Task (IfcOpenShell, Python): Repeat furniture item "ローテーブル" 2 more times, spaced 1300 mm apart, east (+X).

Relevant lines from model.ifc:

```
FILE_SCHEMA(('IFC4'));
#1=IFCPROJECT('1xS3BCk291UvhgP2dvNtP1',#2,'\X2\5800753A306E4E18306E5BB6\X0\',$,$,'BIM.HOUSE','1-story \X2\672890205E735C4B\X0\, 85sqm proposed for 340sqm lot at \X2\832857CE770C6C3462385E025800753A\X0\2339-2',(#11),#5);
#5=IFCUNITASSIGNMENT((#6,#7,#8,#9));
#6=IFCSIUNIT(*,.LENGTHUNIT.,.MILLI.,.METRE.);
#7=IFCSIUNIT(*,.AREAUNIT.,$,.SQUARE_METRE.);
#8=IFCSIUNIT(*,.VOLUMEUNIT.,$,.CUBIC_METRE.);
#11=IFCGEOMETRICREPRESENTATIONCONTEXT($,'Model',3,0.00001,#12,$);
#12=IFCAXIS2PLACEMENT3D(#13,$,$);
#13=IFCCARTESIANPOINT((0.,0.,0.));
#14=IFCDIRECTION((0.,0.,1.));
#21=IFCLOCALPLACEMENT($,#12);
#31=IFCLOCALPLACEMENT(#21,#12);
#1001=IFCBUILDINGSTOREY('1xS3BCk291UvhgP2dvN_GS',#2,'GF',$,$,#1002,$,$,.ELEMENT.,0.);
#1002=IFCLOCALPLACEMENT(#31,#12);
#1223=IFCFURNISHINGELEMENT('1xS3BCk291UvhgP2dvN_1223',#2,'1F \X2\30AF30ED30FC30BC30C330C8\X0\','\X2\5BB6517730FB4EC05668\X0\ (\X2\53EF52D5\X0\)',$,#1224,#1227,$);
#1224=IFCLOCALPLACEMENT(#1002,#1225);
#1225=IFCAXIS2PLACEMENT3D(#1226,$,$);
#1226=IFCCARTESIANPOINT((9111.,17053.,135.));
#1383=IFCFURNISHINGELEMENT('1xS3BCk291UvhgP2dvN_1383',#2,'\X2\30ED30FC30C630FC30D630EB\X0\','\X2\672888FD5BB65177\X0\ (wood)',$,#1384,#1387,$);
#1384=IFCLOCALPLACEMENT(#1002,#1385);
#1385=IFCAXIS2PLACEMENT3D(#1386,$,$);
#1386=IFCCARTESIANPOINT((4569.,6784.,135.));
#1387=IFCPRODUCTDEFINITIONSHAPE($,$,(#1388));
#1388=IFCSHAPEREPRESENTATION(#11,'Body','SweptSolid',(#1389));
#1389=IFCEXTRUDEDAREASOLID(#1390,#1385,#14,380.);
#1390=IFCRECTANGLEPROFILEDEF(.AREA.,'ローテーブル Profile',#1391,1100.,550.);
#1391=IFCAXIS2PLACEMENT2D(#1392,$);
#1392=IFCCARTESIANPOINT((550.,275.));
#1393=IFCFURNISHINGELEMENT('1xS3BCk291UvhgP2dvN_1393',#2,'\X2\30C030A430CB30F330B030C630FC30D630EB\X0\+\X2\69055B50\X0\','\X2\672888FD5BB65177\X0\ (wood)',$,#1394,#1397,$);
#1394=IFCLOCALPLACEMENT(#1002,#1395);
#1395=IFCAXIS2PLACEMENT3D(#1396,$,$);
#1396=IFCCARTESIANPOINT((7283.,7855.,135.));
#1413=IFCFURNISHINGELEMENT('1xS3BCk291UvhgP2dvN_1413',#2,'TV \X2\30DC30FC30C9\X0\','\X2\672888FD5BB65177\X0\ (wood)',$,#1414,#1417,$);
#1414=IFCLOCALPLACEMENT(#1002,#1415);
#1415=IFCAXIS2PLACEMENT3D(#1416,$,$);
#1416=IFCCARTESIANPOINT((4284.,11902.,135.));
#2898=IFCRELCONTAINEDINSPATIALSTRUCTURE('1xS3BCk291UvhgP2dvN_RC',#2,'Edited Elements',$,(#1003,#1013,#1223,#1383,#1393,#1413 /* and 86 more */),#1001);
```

```python
import numpy as np
import ifcopenshell
import ifcopenshell.api.geometry
import ifcopenshell.api.root
import ifcopenshell.util.element
import ifcopenshell.util.placement

model = ifcopenshell.open("model.ifc")


def reuse_history(source, copy):
    """copy_class also copies each property set's owner history, people and application; keep the originals."""
    for rel in copy.IsDefinedBy:
        if rel.is_a("IfcRelDefinesByProperties") and (history := rel.RelatingPropertyDefinition.OwnerHistory):
            rel.RelatingPropertyDefinition.OwnerHistory = source.OwnerHistory
            ifcopenshell.util.element.remove_deep2(model, history)


source = model.by_guid("1xS3BCk291UvhgP2dvN_1383")
base = ifcopenshell.util.placement.get_local_placement(source.ObjectPlacement)
step = np.array([1.0, 0.0, 0.0]) * 1300.0

for i in range(1, 3):
    copy = ifcopenshell.api.root.copy_class(model, product=source)
    copy.Representation = ifcopenshell.util.element.copy_deep(
        model, source.Representation, exclude=["IfcGeometricRepresentationContext", "IfcRepresentationMap"]
    )
    reuse_history(source, copy)
    matrix = base.copy()
    matrix[:3, 3] += i * step
    print("added at", matrix[:3, 3].round(3) + 0.0)
    ifcopenshell.api.geometry.edit_object_placement(model, product=copy, matrix=matrix, is_si=False)

model.write("model_rev.ifc")
```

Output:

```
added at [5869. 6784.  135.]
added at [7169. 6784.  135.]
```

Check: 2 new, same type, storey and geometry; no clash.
